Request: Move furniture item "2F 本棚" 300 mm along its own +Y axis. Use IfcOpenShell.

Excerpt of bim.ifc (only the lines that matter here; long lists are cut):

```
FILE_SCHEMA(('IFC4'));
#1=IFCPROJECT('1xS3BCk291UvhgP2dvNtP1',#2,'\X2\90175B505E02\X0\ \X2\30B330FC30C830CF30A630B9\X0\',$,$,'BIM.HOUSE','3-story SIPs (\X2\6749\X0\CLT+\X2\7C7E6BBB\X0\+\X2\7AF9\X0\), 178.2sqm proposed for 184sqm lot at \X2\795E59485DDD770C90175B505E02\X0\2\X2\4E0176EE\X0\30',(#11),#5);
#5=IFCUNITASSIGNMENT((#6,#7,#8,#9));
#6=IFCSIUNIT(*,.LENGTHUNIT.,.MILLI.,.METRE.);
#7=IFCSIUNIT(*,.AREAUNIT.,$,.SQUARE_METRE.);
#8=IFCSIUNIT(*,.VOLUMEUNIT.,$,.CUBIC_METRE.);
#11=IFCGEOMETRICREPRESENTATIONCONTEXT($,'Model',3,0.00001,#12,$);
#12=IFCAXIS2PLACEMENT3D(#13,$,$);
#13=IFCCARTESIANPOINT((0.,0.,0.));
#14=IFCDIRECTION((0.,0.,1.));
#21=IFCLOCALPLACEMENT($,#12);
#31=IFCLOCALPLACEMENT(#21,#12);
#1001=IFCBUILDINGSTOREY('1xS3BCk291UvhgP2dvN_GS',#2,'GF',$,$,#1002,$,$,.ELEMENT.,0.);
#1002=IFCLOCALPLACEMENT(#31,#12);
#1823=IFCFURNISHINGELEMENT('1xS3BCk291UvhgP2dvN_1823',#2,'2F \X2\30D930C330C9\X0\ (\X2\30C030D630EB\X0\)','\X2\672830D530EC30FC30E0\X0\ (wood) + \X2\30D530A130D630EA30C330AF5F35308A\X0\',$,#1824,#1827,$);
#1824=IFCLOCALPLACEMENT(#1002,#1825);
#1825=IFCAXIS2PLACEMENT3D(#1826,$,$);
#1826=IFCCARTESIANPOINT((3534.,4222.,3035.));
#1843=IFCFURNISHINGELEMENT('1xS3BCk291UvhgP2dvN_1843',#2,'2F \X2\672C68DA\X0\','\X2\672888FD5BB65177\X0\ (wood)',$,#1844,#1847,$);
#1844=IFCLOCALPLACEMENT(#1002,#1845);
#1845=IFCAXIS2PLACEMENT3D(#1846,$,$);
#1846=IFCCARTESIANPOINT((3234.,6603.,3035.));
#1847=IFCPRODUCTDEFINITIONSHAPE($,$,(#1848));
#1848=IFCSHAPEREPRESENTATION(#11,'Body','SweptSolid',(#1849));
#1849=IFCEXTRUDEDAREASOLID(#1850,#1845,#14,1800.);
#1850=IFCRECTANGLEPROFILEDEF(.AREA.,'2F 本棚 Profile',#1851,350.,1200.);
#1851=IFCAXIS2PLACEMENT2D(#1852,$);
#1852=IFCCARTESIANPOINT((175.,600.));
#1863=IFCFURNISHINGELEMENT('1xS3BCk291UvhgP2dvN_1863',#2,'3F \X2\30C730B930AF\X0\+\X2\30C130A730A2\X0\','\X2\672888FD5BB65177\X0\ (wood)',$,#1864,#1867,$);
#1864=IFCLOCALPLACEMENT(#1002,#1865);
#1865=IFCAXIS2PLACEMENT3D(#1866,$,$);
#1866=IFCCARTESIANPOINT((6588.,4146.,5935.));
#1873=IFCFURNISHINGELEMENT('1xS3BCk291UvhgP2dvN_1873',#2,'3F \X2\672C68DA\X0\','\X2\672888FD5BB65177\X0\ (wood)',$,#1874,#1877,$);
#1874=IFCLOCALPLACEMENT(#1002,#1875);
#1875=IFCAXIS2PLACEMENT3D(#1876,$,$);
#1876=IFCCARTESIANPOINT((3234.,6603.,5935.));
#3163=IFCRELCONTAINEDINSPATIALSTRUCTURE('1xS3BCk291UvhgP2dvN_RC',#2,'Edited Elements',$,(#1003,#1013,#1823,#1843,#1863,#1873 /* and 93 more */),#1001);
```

```python
import ifcopenshell
import ifcopenshell.api.geometry
import ifcopenshell.util.placement

model = ifcopenshell.open("bim.ifc")

item = model.by_guid("1xS3BCk291UvhgP2dvN_1843")
matrix = ifcopenshell.util.placement.get_local_placement(item.ObjectPlacement)
matrix[:3, 3] += matrix[:3, 1] * 300.0
ifcopenshell.api.geometry.edit_object_placement(model, product=item, matrix=matrix, is_si=False)

print(ifcopenshell.util.placement.get_local_placement(item.ObjectPlacement).round(3) + 0.0)

model.write("bim-out.ifc")
```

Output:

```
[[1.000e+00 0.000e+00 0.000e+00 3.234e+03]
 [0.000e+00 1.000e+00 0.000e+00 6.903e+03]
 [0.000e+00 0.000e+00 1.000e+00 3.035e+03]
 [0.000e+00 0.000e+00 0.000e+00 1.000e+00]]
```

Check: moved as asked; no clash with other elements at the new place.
